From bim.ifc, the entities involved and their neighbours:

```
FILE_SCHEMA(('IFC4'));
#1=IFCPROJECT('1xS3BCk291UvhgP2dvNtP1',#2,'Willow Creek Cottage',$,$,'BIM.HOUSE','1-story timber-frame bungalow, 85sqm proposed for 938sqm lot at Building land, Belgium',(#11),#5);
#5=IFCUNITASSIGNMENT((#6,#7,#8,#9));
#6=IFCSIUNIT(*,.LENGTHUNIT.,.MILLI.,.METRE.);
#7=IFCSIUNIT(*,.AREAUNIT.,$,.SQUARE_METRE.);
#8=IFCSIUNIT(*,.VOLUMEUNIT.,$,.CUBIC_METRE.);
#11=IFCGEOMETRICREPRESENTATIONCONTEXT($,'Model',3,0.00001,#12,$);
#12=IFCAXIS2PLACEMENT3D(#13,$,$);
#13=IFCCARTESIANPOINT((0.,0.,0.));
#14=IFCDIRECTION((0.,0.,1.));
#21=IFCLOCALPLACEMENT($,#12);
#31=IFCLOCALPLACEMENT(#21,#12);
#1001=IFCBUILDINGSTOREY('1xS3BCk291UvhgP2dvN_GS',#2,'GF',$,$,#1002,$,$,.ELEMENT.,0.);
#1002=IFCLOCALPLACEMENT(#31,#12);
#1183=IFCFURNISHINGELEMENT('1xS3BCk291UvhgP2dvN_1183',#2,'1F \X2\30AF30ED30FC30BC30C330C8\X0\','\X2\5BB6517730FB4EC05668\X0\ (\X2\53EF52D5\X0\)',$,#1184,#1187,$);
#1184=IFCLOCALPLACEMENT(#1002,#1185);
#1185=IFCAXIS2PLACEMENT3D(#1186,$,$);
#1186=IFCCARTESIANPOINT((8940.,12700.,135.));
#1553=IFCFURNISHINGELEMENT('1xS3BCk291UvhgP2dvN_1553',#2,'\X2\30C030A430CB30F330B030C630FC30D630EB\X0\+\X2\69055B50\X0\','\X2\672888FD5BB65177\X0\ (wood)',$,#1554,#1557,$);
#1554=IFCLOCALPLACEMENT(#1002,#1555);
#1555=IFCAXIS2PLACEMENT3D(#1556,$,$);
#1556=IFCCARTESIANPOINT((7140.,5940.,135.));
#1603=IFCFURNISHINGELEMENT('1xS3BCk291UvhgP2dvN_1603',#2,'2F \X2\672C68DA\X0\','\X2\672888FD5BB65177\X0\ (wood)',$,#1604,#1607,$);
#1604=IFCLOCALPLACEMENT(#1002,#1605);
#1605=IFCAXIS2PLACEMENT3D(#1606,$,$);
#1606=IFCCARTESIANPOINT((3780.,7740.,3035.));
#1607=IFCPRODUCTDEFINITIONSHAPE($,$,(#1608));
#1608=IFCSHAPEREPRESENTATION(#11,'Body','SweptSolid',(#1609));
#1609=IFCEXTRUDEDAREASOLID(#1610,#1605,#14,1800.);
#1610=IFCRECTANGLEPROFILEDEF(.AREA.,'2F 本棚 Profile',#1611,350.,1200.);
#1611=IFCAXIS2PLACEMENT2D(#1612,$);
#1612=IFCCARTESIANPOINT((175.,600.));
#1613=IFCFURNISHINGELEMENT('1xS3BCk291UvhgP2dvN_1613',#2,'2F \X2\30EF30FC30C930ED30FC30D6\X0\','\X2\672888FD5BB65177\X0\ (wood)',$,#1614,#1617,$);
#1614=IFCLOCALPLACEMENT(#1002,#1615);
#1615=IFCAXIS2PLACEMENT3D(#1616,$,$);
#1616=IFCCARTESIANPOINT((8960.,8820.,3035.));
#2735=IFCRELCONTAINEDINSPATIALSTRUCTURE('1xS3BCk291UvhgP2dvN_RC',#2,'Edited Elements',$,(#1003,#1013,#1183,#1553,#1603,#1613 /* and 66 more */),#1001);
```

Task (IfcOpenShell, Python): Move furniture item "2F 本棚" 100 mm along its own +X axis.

```python
import ifcopenshell
import ifcopenshell.api.geometry
import ifcopenshell.util.placement

model = ifcopenshell.open("bim.ifc")

item = model.by_guid("1xS3BCk291UvhgP2dvN_1603")
matrix = ifcopenshell.util.placement.get_local_placement(item.ObjectPlacement)
matrix[:3, 3] += matrix[:3, 0] * 100.0
ifcopenshell.api.geometry.edit_object_placement(model, product=item, matrix=matrix, is_si=False)

print(ifcopenshell.util.placement.get_local_placement(item.ObjectPlacement).round(3) + 0.0)

model.write("bim_rev.ifc")
```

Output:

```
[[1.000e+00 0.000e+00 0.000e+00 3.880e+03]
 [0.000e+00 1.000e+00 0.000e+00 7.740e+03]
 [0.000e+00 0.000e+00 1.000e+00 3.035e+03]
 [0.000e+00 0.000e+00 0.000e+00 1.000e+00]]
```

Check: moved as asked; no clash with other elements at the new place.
